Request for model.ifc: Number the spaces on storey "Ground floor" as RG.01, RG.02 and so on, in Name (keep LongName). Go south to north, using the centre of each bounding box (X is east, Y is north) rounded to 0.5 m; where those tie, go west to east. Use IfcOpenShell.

First a look at what the model holds.

```python
import ifcopenshell
import ifcopenshell.util.element
import ifcopenshell.util.placement

model = ifcopenshell.open("model.ifc")
print(model.schema)
storey = next(s for s in model.by_type("IfcBuildingStorey") if s.Name == "Ground floor")
spaces = [e for e in ifcopenshell.util.element.get_decomposition(storey) if e.is_a("IfcSpace")]
for e in sorted(spaces, key=lambda e: e.id()):
    origin = ifcopenshell.util.placement.get_local_placement(e.ObjectPlacement)[:3, 3]
    print(e.id(), e.Name, e.LongName, origin.round(2) + 0.0, sep=" | ")
```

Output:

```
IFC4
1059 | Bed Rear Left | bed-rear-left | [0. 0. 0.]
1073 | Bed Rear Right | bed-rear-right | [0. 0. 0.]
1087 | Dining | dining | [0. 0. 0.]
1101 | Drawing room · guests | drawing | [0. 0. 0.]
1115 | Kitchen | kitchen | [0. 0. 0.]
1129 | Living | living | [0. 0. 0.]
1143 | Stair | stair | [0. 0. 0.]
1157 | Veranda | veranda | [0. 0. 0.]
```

```python
import ifcopenshell
import ifcopenshell.geom
import ifcopenshell.util.element
import ifcopenshell.util.shape

model = ifcopenshell.open("model.ifc")
settings = ifcopenshell.geom.settings()
settings.set("use-world-coords", True)


def centre(element):
    shape = ifcopenshell.geom.create_shape(settings, element)
    return ifcopenshell.util.shape.get_bbox_centroid(shape.geometry)


storey = next(s for s in model.by_type("IfcBuildingStorey") if s.Name == "Ground floor")
spaces = [e for e in ifcopenshell.util.element.get_decomposition(storey) if e.is_a("IfcSpace")]

# Insertion points can sit at a corner or the storey origin, so sort by the geometry (in metres).
centres = {e: centre(e) for e in spaces}
spaces.sort(key=lambda e: (round(centres[e][1] / 0.5), centres[e][0]))

for i, e in enumerate(spaces, start=1):
    number = f"RG.{i:02d}"
    e.Name = number
    print(e.id(), number)

model.write("model_edited.ifc")
```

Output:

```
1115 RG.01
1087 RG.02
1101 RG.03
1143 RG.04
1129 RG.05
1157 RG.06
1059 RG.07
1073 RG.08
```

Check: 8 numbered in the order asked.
